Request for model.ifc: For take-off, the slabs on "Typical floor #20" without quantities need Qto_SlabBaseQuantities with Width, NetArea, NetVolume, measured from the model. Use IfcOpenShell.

First a look at what the model holds.

```python
import ifcopenshell
import ifcopenshell.util.element
import ifcopenshell.util.unit

model = ifcopenshell.open("model.ifc")
print(model.schema)
for unit_type in ("LENGTHUNIT", "AREAUNIT", "VOLUMEUNIT"):
    print(unit_type, ifcopenshell.util.unit.calculate_unit_scale(model, unit_type))
storey = next(s for s in model.by_type("IfcBuildingStorey") if s.Name == "Typical floor #20")
slabs = [e for e in ifcopenshell.util.element.get_decomposition(storey) if e.is_a("IfcSlab")]
for e in sorted(slabs, key=lambda e: e.id()):
    print(e.id(), e.is_a(), e.Name, list(ifcopenshell.util.element.get_psets(e, qtos_only=True)), sep=" | ")
```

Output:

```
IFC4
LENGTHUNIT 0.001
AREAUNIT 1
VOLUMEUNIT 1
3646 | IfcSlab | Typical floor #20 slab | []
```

```python
import ifcopenshell
import ifcopenshell.api.pset
import ifcopenshell.geom
import ifcopenshell.util.element
import ifcopenshell.util.shape
import ifcopenshell.util.unit

model = ifcopenshell.open("model.ifc")
unit_scale = ifcopenshell.util.unit.calculate_unit_scale(model)
area_scale = ifcopenshell.util.unit.calculate_unit_scale(model, "AREAUNIT")
volume_scale = ifcopenshell.util.unit.calculate_unit_scale(model, "VOLUMEUNIT")
settings = ifcopenshell.geom.settings()

storey = next(s for s in model.by_type("IfcBuildingStorey") if s.Name == "Typical floor #20")
slabs = [e for e in ifcopenshell.util.element.get_decomposition(storey) if e.is_a("IfcSlab")]

for e in sorted(slabs, key=lambda e: e.id()):
    if ifcopenshell.util.element.get_psets(e, qtos_only=True, should_inherit=False):
        continue
    # Geometry comes back in metres, in the element's own axes.
    shape = ifcopenshell.geom.create_shape(settings, e)
    values = {
        "Width": ifcopenshell.util.shape.get_z(shape.geometry) / unit_scale,
        "NetArea": ifcopenshell.util.shape.get_footprint_area(shape.geometry) / area_scale,
        "NetVolume": ifcopenshell.util.shape.get_volume(shape.geometry) / volume_scale,
    }
    qto = ifcopenshell.api.pset.add_qto(model, product=e, name="Qto_SlabBaseQuantities")
    ifcopenshell.api.pset.edit_qto(model, qto=qto, properties=values)
    print(e.id(), {k: round(v, 3) for k, v in values.items()})

model.write("model_updated.ifc")
```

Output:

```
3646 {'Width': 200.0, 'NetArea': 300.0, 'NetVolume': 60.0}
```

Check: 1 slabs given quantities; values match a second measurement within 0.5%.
